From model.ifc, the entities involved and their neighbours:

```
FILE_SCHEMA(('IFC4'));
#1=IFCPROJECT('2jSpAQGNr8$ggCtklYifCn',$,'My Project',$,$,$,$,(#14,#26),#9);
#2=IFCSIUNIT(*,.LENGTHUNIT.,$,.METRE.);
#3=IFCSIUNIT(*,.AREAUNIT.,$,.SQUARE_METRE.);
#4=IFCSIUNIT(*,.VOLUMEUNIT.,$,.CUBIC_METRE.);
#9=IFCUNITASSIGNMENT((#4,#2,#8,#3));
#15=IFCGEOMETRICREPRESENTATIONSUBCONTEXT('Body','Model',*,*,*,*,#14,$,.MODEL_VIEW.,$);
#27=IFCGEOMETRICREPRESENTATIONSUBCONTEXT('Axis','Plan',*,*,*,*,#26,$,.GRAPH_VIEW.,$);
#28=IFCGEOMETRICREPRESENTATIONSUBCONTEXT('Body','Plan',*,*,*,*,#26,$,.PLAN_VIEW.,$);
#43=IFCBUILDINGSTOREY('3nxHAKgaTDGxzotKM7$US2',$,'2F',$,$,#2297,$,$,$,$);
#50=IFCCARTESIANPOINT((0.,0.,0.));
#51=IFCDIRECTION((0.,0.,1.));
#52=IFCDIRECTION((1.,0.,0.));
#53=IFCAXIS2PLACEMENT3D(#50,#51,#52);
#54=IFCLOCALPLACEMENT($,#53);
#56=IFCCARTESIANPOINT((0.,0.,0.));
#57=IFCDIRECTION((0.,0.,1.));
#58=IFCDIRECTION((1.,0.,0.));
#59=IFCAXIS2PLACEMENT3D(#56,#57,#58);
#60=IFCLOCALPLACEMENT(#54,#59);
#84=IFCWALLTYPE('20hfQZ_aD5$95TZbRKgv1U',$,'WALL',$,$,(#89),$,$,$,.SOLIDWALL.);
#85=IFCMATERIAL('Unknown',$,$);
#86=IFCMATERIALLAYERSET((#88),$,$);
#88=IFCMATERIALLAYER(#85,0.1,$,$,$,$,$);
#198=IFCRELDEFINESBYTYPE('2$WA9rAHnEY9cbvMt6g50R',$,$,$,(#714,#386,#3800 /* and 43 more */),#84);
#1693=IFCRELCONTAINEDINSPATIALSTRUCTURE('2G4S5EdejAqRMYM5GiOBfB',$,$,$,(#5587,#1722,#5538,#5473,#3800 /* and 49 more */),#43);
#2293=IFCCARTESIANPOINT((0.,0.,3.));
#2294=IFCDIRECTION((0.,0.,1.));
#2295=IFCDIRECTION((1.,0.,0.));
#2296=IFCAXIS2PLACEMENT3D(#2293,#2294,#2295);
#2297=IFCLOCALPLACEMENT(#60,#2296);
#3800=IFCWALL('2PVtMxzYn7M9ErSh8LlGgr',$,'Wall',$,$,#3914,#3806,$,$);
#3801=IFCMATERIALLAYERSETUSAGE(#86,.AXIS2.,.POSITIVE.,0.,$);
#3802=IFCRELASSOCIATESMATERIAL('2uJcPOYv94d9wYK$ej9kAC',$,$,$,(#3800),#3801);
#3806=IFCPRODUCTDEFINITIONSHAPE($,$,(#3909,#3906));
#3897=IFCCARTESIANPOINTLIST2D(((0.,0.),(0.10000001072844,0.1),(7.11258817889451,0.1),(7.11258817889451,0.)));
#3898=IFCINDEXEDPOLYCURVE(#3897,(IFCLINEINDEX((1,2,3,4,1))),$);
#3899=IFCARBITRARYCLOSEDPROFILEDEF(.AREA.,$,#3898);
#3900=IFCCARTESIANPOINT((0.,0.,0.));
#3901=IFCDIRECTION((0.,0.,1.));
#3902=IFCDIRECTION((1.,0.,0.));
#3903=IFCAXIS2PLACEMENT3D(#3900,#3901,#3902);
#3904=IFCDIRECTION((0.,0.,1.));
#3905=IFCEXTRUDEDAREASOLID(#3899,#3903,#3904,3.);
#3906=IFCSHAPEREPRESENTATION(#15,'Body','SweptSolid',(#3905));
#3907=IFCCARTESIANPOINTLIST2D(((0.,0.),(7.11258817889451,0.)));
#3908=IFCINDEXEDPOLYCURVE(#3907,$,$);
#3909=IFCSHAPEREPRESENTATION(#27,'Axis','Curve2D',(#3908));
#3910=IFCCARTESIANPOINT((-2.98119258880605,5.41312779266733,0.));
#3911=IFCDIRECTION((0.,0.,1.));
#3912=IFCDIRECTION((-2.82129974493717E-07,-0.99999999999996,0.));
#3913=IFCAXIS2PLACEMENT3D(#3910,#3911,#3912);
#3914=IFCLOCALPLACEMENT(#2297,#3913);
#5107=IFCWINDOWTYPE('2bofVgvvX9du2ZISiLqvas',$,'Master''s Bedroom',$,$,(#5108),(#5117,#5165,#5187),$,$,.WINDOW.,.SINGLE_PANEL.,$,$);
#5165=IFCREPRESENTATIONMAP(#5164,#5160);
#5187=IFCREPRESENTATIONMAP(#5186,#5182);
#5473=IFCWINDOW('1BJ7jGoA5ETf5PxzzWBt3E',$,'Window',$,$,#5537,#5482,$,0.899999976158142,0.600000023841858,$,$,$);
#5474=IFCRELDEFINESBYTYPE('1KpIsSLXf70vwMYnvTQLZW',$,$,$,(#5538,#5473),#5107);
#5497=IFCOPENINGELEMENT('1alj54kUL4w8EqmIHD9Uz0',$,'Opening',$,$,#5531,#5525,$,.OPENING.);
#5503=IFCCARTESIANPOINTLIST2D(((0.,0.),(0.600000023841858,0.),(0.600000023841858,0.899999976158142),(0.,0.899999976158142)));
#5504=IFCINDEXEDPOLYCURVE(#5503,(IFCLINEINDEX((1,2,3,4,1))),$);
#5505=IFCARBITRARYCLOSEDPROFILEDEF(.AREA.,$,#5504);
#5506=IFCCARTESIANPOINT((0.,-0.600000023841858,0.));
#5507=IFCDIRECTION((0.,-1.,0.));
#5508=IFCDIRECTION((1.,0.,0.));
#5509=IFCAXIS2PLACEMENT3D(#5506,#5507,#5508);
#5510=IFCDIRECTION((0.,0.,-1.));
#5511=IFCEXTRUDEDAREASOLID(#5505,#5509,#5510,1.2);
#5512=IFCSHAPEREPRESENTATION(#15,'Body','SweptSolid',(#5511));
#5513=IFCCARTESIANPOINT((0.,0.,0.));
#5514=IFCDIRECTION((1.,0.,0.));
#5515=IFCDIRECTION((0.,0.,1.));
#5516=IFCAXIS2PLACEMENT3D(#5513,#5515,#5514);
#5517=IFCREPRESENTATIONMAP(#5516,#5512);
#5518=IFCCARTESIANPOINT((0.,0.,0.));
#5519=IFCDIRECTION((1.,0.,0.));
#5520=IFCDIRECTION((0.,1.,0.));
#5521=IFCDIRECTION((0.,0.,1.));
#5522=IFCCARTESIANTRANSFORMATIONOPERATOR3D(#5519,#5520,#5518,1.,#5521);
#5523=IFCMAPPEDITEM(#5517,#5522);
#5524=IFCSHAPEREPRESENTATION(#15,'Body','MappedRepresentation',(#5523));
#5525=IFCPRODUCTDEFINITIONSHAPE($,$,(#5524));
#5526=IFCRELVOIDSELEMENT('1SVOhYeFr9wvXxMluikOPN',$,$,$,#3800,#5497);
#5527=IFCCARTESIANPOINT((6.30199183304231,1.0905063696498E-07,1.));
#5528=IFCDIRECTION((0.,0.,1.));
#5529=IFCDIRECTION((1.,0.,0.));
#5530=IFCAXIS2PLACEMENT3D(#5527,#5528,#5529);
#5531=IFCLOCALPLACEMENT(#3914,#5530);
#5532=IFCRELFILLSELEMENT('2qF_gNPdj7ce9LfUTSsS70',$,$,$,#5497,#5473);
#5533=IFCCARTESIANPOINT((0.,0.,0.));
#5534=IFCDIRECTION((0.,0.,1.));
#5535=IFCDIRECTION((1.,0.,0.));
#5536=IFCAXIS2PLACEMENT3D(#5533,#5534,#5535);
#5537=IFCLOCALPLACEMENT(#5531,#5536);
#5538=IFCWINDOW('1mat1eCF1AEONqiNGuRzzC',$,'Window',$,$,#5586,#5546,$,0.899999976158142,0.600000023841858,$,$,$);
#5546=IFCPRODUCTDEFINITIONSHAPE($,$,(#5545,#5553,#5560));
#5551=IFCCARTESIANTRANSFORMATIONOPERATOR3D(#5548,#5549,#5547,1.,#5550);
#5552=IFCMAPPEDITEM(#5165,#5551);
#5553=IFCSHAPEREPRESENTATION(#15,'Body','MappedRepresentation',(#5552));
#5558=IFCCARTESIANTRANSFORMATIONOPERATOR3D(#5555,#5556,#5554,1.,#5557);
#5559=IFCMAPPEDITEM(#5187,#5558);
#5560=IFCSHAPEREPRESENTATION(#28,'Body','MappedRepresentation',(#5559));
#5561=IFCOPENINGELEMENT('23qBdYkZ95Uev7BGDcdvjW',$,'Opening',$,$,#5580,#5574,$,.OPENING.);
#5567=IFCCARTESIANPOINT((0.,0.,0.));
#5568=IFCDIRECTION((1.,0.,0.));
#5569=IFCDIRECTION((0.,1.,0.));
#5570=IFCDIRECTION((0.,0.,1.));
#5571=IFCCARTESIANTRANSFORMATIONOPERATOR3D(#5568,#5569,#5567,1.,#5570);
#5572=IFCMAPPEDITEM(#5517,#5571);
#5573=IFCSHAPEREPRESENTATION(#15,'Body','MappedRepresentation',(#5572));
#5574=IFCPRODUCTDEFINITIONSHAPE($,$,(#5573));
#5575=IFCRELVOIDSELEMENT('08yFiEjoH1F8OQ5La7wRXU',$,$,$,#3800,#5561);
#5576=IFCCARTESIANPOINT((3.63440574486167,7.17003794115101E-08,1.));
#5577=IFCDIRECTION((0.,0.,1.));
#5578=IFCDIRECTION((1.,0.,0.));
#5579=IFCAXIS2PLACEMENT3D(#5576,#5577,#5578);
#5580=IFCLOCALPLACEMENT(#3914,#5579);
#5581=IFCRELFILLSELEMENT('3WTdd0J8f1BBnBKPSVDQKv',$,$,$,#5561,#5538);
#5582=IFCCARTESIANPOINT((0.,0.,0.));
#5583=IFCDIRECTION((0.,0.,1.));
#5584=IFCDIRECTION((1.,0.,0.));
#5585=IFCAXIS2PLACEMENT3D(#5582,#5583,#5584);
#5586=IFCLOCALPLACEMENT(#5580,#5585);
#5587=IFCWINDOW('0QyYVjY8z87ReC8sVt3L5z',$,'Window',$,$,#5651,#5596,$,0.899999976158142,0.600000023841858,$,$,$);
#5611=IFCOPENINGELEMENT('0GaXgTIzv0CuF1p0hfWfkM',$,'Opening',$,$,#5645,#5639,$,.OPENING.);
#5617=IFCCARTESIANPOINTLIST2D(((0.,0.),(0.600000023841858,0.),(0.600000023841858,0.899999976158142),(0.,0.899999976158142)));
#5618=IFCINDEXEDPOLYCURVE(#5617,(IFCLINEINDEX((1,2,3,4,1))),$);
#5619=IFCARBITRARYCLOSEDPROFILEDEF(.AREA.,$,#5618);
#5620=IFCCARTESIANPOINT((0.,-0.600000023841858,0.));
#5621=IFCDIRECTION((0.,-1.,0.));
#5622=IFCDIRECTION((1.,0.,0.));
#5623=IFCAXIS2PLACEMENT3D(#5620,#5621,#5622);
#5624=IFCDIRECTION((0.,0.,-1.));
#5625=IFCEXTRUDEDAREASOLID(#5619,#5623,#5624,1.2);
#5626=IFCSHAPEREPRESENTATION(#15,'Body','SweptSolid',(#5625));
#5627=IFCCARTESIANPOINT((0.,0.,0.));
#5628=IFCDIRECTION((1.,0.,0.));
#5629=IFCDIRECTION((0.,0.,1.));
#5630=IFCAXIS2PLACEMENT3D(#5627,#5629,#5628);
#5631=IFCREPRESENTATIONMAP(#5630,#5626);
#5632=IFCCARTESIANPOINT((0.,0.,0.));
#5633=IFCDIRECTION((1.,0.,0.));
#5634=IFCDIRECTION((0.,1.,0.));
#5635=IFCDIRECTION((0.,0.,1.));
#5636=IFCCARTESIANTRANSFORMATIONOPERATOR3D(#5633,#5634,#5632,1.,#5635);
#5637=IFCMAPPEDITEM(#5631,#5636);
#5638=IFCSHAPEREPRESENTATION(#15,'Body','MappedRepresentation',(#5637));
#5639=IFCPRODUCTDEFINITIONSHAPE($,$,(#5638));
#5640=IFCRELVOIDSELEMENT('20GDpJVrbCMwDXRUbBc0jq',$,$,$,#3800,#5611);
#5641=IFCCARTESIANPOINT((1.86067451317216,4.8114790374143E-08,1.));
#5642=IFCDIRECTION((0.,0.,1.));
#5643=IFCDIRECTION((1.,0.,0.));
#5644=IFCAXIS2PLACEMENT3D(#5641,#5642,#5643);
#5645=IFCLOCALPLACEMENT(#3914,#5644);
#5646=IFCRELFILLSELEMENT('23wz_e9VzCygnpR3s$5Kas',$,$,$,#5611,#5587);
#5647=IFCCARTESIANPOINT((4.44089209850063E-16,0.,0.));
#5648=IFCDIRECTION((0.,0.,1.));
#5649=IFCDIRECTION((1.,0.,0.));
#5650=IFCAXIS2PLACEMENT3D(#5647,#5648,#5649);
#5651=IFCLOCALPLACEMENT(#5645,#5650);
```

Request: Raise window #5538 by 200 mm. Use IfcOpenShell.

```python
import numpy as np
import ifcopenshell
import ifcopenshell.api.geometry
import ifcopenshell.util.placement
import ifcopenshell.util.unit

model = ifcopenshell.open("model.ifc")
unit_scale = ifcopenshell.util.unit.calculate_unit_scale(model)

window = model.by_guid("1mat1eCF1AEONqiNGuRzzC")
opening = window.FillsVoids[0].RelatingOpeningElement
dz = 0.2 / unit_scale

shift = np.array([0.0, 0.0, dz])
# The window is placed relative to its opening, so it follows when the opening moves.
matrix = ifcopenshell.util.placement.get_local_placement(opening.ObjectPlacement)
matrix[:3, 3] += shift
ifcopenshell.api.geometry.edit_object_placement(
    model, product=opening, matrix=matrix, is_si=False, should_transform_children=True
)

print(f"moved by {dz * unit_scale:+.3f} m")

model.write("model_v2.ifc")
```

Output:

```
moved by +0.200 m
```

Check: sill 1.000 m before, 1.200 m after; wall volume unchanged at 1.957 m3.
